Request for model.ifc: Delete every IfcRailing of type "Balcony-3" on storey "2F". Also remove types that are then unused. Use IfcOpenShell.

First a look at what the model holds.

```python
import ifcopenshell
import ifcopenshell.util.element

model = ifcopenshell.open("model.ifc")
print(model.schema)
storey = next(s for s in model.by_type("IfcBuildingStorey") if s.Name == "2F")
railings = [e for e in ifcopenshell.util.element.get_decomposition(storey) if e.is_a("IfcRailing")]
seen = {}
for e in railings:
    element_type = ifcopenshell.util.element.get_type(e)
    name = element_type.Name if element_type not in (None, e) else None
    seen[name] = seen.get(name, 0) + 1
for name, count in sorted(seen.items(), key=str):
    print(count, "x", name)
```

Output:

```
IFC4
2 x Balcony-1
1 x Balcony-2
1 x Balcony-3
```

```python
import ifcopenshell
import ifcopenshell.api.root
import ifcopenshell.util.element

model = ifcopenshell.open("model.ifc")

storey = next(s for s in model.by_type("IfcBuildingStorey") if s.Name == "2F")
railings = [e for e in ifcopenshell.util.element.get_decomposition(storey) if e.is_a("IfcRailing")]
targets = [e for e in railings if (t := ifcopenshell.util.element.get_type(e)) not in (None, e) and t.Name == "Balcony-3"]
types = {ifcopenshell.util.element.get_type(e) for e in targets} - {None, *targets}

for e in targets:
    ifcopenshell.api.root.remove_product(model, product=e)
print(len(targets), "removed")

unused = [t for t in types if not ifcopenshell.util.element.get_types(t)]
for t in unused:
    ifcopenshell.api.root.remove_product(model, product=t)
print(len(unused), "unused types removed")

model.write("model_rev.ifc")
```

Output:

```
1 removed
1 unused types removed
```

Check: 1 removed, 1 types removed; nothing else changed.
